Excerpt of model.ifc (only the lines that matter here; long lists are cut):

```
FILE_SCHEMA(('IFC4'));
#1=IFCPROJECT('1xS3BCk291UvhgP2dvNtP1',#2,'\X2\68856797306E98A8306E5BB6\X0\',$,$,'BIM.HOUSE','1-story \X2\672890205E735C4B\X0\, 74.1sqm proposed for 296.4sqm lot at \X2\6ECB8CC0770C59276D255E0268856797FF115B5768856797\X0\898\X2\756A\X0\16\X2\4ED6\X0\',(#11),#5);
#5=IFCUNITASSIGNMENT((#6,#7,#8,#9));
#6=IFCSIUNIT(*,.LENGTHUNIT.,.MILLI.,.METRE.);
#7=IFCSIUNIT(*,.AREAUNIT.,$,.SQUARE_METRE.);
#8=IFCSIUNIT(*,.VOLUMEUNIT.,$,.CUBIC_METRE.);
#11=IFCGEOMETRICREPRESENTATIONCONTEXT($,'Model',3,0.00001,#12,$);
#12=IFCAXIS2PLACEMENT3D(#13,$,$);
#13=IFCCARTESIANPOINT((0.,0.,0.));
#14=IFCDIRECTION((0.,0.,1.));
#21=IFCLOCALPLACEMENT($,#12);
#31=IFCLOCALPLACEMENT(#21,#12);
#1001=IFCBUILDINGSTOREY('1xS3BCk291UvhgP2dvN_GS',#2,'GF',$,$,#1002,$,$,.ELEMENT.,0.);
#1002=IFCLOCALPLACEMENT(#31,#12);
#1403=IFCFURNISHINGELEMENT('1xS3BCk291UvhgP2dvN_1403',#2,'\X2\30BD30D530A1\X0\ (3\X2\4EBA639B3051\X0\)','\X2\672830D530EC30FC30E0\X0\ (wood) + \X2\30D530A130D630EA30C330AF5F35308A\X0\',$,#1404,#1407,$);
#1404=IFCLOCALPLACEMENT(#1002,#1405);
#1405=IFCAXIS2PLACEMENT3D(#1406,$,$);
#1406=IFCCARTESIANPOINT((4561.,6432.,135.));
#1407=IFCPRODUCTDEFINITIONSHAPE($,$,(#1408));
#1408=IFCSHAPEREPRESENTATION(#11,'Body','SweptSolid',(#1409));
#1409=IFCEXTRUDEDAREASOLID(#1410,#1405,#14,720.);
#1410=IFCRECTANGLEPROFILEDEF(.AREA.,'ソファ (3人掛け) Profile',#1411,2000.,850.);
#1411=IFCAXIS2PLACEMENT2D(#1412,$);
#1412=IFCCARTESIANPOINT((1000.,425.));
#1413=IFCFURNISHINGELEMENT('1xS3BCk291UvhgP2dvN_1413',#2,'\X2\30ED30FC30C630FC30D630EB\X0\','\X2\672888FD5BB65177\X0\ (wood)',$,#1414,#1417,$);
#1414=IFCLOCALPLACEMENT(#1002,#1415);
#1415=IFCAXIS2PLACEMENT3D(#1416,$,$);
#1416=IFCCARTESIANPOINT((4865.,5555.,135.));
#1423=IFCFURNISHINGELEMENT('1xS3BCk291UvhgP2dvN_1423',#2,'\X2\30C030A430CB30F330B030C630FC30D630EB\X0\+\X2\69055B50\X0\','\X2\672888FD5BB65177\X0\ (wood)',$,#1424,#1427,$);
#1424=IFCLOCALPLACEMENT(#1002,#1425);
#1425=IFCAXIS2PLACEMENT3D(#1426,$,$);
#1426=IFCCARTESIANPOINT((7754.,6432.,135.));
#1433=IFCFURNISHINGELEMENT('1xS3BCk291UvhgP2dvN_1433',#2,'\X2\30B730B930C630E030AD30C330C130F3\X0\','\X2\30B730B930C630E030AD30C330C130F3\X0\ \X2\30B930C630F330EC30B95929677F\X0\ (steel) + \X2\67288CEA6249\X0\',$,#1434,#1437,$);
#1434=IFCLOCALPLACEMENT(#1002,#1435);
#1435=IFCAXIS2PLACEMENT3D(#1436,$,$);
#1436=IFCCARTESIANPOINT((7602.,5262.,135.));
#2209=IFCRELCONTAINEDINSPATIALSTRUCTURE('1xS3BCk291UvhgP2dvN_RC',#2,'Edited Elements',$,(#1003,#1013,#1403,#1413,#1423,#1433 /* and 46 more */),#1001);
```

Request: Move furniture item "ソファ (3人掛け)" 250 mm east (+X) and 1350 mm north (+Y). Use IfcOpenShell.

```python
import ifcopenshell
import ifcopenshell.api.geometry
import ifcopenshell.util.placement

model = ifcopenshell.open("model.ifc")

item = model.by_guid("1xS3BCk291UvhgP2dvN_1403")
matrix = ifcopenshell.util.placement.get_local_placement(item.ObjectPlacement)
matrix[0, 3] += 250.0
matrix[1, 3] += 1350.0
ifcopenshell.api.geometry.edit_object_placement(model, product=item, matrix=matrix, is_si=False)

print(ifcopenshell.util.placement.get_local_placement(item.ObjectPlacement).round(3) + 0.0)

model.write("model_edited.ifc")
```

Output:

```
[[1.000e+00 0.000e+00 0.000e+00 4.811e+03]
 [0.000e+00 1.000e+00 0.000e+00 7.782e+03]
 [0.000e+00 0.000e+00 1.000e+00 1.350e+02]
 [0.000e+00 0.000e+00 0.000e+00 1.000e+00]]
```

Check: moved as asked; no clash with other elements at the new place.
